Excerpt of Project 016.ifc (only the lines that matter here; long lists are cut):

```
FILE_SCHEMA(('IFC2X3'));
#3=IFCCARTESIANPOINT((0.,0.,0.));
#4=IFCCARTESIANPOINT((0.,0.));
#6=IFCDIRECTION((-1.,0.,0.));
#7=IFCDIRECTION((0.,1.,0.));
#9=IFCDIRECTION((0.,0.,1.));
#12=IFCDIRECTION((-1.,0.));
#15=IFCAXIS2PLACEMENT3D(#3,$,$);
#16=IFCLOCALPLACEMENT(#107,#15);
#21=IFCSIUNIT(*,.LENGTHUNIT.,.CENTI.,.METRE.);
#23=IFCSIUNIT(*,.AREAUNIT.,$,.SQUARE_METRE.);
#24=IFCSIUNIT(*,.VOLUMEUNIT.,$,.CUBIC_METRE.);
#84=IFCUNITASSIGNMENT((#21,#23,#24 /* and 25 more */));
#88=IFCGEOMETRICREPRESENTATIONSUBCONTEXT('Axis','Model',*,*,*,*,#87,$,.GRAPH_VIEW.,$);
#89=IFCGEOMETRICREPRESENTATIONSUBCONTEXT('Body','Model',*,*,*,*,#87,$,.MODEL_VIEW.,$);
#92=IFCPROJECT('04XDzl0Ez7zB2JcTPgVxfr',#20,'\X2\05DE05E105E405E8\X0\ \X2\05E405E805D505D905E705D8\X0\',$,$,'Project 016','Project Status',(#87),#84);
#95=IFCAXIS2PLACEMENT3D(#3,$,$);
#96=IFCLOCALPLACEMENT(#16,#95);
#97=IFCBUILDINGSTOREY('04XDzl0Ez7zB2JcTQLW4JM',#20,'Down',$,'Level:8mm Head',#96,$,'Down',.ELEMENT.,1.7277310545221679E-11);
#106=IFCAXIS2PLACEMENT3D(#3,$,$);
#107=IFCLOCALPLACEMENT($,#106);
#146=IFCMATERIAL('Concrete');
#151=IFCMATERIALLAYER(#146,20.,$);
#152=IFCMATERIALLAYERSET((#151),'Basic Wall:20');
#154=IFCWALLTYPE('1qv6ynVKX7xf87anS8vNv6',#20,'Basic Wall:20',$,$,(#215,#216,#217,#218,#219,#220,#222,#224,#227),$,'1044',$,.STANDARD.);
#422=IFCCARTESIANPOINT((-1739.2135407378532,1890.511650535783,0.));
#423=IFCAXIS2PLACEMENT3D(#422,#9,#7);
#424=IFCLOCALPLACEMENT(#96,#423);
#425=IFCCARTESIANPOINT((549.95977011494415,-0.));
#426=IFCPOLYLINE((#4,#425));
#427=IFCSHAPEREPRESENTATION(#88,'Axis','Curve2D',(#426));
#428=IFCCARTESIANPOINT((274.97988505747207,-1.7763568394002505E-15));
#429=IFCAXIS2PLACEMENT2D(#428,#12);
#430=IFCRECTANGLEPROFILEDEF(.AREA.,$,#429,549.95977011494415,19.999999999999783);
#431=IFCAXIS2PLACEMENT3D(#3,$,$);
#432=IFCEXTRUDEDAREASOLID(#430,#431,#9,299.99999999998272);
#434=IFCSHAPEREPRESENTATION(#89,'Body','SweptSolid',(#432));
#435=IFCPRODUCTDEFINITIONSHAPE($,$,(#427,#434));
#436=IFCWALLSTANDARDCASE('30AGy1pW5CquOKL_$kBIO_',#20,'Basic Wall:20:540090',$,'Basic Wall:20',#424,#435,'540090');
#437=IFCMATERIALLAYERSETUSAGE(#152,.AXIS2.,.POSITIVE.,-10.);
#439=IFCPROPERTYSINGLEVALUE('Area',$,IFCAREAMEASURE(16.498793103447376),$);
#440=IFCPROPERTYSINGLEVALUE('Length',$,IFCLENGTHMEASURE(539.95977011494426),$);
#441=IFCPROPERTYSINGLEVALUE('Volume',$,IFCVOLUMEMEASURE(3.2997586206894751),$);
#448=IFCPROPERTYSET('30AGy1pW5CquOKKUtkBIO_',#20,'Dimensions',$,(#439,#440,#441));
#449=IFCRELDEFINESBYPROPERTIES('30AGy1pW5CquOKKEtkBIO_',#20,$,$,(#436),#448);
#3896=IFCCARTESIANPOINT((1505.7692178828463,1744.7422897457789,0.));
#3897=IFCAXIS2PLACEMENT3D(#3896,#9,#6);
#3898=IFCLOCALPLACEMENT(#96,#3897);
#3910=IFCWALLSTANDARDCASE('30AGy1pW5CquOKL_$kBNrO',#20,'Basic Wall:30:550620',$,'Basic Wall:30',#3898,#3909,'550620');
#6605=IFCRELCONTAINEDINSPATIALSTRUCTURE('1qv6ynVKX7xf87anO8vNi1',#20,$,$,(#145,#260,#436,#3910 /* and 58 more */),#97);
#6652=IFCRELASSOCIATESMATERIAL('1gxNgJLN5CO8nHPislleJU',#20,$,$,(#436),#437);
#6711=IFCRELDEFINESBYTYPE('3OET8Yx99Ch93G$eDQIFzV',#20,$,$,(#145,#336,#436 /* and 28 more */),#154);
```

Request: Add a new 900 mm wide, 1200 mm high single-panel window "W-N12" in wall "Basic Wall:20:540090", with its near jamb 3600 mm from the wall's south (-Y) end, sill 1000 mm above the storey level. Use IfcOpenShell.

```python
import numpy as np
import ifcopenshell
import ifcopenshell.api.feature
import ifcopenshell.api.geometry
import ifcopenshell.api.pset
import ifcopenshell.api.root
import ifcopenshell.api.spatial
import ifcopenshell.api.type
import ifcopenshell.geom
import ifcopenshell.util.element
import ifcopenshell.util.placement
import ifcopenshell.util.representation
import ifcopenshell.util.shape
import ifcopenshell.util.unit

model = ifcopenshell.open("Project 016.ifc")
unit_scale = ifcopenshell.util.unit.calculate_unit_scale(model)
area_scale = ifcopenshell.util.unit.calculate_unit_scale(model, "AREAUNIT")
volume_scale = ifcopenshell.util.unit.calculate_unit_scale(model, "VOLUMEUNIT")
settings = ifcopenshell.geom.settings()


def volume(element):
    """Net volume in cubic metres, openings subtracted."""
    shape = ifcopenshell.geom.create_shape(settings, element)
    return ifcopenshell.util.shape.get_volume(shape.geometry)


wall = model.by_guid("30AGy1pW5CquOKL_$kBIO_")
storey = ifcopenshell.util.element.get_container(wall, ifc_class="IfcBuildingStorey")
context = ifcopenshell.util.representation.get_context(model, "Model", "Body", "MODEL_VIEW")
before = volume(wall)

width, height, from_end, sill = 0.9, 1.2, 3.6, 1  # metres

# The wall runs along its own X axis, and the end named is its -X end.
wall_shape = ifcopenshell.geom.create_shape(settings, wall)
x, y, z = ifcopenshell.util.shape.get_vertices(wall_shape.geometry).T
start = x.min() + from_end
face, thickness = float(y.min()), float(y.max() - y.min())
wall_matrix = ifcopenshell.util.placement.get_local_placement(wall.ObjectPlacement)
level = ifcopenshell.util.placement.get_local_placement(storey.ObjectPlacement)[2, 3]


def in_wall(x, y):
    """Placement at x, y metres in the wall's axes, at sill height."""
    matrix = wall_matrix.copy()
    matrix[:, 3] = wall_matrix @ np.array([x / unit_scale, y / unit_scale, 0.0, 1.0])
    matrix[2, 3] = level + sill / unit_scale
    return matrix


# Opening: a box that overshoots both wall faces by 50 mm.
opening = ifcopenshell.api.root.create_entity(model, ifc_class="IfcOpeningElement")
box = ifcopenshell.api.geometry.add_wall_representation(
    model, context=context, length=width, height=height, thickness=thickness + 0.1
)
ifcopenshell.api.geometry.assign_representation(model, product=opening, representation=box)
ifcopenshell.api.geometry.edit_object_placement(model, product=opening, matrix=in_wall(start, face - 0.05), is_si=False)
ifcopenshell.api.feature.add_feature(model, feature=opening, element=wall)

window = ifcopenshell.api.root.create_entity(model, ifc_class="IfcWindow", name="W-N12")
window.OverallWidth, window.OverallHeight = width / unit_scale, height / unit_scale
body = ifcopenshell.api.geometry.add_window_representation(
    model,
    context=context,
    overall_width=window.OverallWidth,
    overall_height=window.OverallHeight,
    partition_type="SINGLE_PANEL",
)
ifcopenshell.api.geometry.assign_representation(model, product=window, representation=body)
ifcopenshell.api.spatial.assign_container(model, products=[window], relating_structure=storey)
fills = ifcopenshell.api.feature.add_filling(model, opening=opening, element=window)
fills.OwnerHistory = window.OwnerHistory  # required in IFC2X3

# IFC2X3 keeps the operation on the window style.
style = ifcopenshell.api.root.create_entity(model, ifc_class="IfcWindowStyle", name="W-N12")
style.OperationType, style.ConstructionType = "SINGLE_PANEL", "NOTDEFINED"
style.ParameterTakesPrecedence = style.Sizeable = False
ifcopenshell.api.type.assign_type(model, related_objects=[window], relating_type=style)

# Centre the window in the wall's thickness.
ifcopenshell.api.geometry.edit_object_placement(model, product=window, matrix=in_wall(start, face), is_si=False)
window_shape = ifcopenshell.geom.create_shape(settings, window)
depth = ifcopenshell.util.shape.get_vertices(window_shape.geometry)[:, 1]
offset = face + thickness / 2 - (depth.min() + depth.max()) / 2
ifcopenshell.api.geometry.edit_object_placement(model, product=window, matrix=in_wall(start, offset), is_si=False)

after = volume(wall)

# Update the wall's stored quantities.
pset = model.by_id(ifcopenshell.util.element.get_pset(wall, "Dimensions", should_inherit=False)["id"])
ifcopenshell.api.pset.edit_pset(model, pset=pset, properties={
    "Area": model.create_entity("IfcAreaMeasure", after / thickness / area_scale),
    "Volume": model.create_entity("IfcVolumeMeasure", after / volume_scale),
})

print(f"wall volume {before:.3f} -> {after:.3f} m3")

model.write("Project 016-out.ifc")
```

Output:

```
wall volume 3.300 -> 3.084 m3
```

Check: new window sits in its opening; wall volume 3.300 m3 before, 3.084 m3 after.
